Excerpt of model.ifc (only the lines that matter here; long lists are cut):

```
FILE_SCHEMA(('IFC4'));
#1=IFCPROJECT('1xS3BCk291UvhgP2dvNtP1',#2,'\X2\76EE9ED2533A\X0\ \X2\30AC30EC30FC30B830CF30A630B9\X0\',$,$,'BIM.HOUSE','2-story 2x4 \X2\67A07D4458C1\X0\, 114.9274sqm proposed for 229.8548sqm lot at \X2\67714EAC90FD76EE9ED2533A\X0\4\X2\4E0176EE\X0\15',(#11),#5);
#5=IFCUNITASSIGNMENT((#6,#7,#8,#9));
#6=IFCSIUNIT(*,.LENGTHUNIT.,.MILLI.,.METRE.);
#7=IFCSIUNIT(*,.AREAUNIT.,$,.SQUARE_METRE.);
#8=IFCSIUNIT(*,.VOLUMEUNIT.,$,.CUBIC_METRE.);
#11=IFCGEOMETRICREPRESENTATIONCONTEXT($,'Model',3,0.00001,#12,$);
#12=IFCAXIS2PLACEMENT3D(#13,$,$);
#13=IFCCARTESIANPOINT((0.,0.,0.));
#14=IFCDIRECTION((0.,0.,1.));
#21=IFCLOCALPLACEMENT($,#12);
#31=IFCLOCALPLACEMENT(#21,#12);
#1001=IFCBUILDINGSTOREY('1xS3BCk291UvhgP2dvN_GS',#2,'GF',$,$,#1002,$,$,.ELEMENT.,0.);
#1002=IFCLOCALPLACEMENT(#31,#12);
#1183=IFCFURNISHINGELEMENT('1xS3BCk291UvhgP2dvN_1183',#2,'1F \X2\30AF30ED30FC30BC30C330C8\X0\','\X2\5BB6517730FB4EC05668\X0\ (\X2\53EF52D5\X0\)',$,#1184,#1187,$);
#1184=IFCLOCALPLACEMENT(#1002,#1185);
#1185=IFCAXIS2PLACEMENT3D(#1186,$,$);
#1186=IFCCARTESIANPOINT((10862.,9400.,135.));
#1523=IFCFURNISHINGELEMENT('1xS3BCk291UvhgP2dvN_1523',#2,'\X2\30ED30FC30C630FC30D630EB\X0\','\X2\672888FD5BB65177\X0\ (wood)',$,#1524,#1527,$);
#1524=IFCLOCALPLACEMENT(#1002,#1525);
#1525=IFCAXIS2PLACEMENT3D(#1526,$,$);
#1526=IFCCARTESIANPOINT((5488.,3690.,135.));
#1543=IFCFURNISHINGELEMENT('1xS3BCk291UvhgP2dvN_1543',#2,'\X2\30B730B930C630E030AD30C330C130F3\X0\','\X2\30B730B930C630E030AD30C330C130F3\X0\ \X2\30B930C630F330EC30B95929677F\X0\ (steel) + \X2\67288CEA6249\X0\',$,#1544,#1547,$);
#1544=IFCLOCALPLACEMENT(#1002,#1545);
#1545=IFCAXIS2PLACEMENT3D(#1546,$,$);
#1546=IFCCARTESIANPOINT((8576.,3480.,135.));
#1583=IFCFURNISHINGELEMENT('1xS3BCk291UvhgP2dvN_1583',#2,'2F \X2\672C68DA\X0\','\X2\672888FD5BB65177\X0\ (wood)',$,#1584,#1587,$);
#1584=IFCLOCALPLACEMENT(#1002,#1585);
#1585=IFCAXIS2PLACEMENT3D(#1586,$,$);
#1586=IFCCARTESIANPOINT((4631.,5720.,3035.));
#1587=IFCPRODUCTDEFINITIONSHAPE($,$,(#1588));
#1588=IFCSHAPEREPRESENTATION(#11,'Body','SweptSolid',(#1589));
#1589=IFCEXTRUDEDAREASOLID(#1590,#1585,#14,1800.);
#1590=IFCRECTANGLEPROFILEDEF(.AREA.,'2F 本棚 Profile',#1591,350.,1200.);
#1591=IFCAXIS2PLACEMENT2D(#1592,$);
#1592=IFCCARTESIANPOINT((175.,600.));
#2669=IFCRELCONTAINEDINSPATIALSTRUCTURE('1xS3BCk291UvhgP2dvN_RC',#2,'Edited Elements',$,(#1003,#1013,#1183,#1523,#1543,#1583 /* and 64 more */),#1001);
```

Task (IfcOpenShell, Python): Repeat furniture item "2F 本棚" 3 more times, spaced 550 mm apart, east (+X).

```python
import numpy as np
import ifcopenshell
import ifcopenshell.api.geometry
import ifcopenshell.api.root
import ifcopenshell.util.element
import ifcopenshell.util.placement
import ifcopenshell.util.unit

model = ifcopenshell.open("model.ifc")
unit_scale = ifcopenshell.util.unit.calculate_unit_scale(model)


def reuse_history(source, copy):
    """copy_class also copies each property set's owner history, people and application; keep the originals."""
    for rel in copy.IsDefinedBy:
        if rel.is_a("IfcRelDefinesByProperties") and (history := rel.RelatingPropertyDefinition.OwnerHistory):
            rel.RelatingPropertyDefinition.OwnerHistory = source.OwnerHistory
            ifcopenshell.util.element.remove_deep2(model, history)


source = model.by_guid("1xS3BCk291UvhgP2dvN_1583")
base = ifcopenshell.util.placement.get_local_placement(source.ObjectPlacement)
step = np.array([1.0, 0.0, 0.0]) * 0.55 / unit_scale

for i in range(1, 4):
    copy = ifcopenshell.api.root.copy_class(model, product=source)
    copy.Representation = ifcopenshell.util.element.copy_deep(
        model, source.Representation, exclude=["IfcGeometricRepresentationContext", "IfcRepresentationMap"]
    )
    reuse_history(source, copy)
    matrix = base.copy()
    matrix[:3, 3] += i * step
    print("added at", matrix[:3, 3].round(3) + 0.0)
    ifcopenshell.api.geometry.edit_object_placement(model, product=copy, matrix=matrix, is_si=False)

model.write("model_rev.ifc")
```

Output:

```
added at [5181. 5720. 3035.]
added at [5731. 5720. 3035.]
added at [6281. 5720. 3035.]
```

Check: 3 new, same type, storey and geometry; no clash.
